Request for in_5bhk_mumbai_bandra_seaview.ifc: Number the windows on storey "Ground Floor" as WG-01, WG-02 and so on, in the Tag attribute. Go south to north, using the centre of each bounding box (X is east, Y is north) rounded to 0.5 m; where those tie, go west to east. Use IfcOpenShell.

First a look at what the model holds.

```python
import ifcopenshell
import ifcopenshell.util.element
import ifcopenshell.util.placement

model = ifcopenshell.open("in_5bhk_mumbai_bandra_seaview.ifc")
print(model.schema)
storey = next(s for s in model.by_type("IfcBuildingStorey") if s.Name == "Ground Floor")
windows = [e for e in ifcopenshell.util.element.get_decomposition(storey) if e.is_a("IfcWindow")]
for e in sorted(windows, key=lambda e: e.id()):
    origin = ifcopenshell.util.placement.get_local_placement(e.ObjectPlacement)[:3, 3]
    print(e.id(), e.Tag, e.Name, origin.round(2) + 0.0, sep=" | ")
```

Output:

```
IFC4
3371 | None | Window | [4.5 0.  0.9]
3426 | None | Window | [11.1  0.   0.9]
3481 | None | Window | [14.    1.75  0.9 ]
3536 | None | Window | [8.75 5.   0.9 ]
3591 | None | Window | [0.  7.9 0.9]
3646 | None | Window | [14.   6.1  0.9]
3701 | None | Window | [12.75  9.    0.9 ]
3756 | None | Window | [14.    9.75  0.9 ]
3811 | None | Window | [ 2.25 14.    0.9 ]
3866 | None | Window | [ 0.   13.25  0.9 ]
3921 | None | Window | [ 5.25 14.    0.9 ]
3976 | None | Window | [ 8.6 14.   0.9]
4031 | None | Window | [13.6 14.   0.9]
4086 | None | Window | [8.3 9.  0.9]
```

```python
import ifcopenshell
import ifcopenshell.geom
import ifcopenshell.util.element
import ifcopenshell.util.shape

model = ifcopenshell.open("in_5bhk_mumbai_bandra_seaview.ifc")
settings = ifcopenshell.geom.settings()
settings.set("use-world-coords", True)


def centre(element):
    shape = ifcopenshell.geom.create_shape(settings, element)
    return ifcopenshell.util.shape.get_bbox_centroid(shape.geometry)


storey = next(s for s in model.by_type("IfcBuildingStorey") if s.Name == "Ground Floor")
windows = [e for e in ifcopenshell.util.element.get_decomposition(storey) if e.is_a("IfcWindow")]

# Insertion points can sit at a corner or the storey origin, so sort by the geometry (in metres).
centres = {e: centre(e) for e in windows}
windows.sort(key=lambda e: (round(centres[e][1] / 0.5), centres[e][0]))

for i, e in enumerate(windows, start=1):
    number = f"WG-{i:02d}"
    e.Tag = number
    print(e.id(), number)

model.write("in_5bhk_mumbai_bandra_seaview_updated.ifc")
```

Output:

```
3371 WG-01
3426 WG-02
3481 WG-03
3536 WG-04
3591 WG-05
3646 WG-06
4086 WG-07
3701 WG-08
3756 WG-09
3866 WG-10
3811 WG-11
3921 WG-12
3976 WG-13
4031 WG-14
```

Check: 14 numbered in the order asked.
